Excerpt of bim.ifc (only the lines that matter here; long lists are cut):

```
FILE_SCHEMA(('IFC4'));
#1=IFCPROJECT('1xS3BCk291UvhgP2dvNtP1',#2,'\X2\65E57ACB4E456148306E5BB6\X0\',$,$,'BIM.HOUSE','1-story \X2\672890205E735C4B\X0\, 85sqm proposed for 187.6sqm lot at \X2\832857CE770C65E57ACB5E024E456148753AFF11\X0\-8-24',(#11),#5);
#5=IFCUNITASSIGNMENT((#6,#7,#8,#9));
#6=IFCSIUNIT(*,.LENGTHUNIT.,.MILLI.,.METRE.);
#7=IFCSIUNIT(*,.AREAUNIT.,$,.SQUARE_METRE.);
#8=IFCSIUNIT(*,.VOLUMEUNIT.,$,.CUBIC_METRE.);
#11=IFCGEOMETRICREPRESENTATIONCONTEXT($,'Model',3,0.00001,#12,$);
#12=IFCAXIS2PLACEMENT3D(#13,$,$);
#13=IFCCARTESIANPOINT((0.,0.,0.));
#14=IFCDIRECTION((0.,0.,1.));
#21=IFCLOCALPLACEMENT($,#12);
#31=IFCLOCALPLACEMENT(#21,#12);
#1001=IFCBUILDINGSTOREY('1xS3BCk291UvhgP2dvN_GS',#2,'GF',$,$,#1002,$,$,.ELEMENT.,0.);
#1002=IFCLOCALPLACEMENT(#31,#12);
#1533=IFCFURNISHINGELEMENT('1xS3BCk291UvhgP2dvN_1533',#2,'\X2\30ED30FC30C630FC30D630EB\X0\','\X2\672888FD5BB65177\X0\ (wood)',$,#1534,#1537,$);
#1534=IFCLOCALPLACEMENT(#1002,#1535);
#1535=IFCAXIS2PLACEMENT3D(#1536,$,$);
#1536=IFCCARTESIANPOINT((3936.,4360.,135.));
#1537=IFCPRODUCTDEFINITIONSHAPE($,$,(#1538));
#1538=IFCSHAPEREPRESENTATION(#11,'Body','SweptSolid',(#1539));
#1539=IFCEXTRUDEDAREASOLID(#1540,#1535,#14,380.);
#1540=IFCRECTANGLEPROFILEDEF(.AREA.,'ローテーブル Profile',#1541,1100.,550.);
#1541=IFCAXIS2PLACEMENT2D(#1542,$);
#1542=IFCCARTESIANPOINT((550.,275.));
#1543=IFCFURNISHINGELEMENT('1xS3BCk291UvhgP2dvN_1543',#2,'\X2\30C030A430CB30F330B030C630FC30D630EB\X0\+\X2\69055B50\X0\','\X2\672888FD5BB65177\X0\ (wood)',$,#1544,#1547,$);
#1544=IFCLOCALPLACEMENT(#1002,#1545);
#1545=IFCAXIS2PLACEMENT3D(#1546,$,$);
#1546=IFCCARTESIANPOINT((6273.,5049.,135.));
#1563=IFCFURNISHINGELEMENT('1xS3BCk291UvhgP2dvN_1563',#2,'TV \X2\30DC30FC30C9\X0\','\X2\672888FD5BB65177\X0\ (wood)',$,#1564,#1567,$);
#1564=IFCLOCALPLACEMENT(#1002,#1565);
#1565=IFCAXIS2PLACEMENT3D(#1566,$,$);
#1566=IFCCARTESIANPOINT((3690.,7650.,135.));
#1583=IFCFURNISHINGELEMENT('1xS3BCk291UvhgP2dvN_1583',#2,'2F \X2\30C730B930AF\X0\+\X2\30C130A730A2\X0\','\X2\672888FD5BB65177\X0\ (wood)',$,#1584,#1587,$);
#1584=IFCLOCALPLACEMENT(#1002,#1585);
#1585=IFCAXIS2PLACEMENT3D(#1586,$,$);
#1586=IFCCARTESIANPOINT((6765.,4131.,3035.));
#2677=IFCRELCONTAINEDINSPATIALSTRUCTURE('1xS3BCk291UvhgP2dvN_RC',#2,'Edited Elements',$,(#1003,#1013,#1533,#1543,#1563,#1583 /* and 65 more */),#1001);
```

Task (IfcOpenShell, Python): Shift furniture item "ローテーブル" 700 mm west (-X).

```python
import ifcopenshell
import ifcopenshell.api.geometry
import ifcopenshell.util.placement
import ifcopenshell.util.unit

model = ifcopenshell.open("bim.ifc")
unit_scale = ifcopenshell.util.unit.calculate_unit_scale(model)

item = model.by_guid("1xS3BCk291UvhgP2dvN_1533")
matrix = ifcopenshell.util.placement.get_local_placement(item.ObjectPlacement)
matrix[0, 3] -= 0.7 / unit_scale
ifcopenshell.api.geometry.edit_object_placement(model, product=item, matrix=matrix, is_si=False)

print(ifcopenshell.util.placement.get_local_placement(item.ObjectPlacement).round(3) + 0.0)

model.write("bim-out.ifc")
```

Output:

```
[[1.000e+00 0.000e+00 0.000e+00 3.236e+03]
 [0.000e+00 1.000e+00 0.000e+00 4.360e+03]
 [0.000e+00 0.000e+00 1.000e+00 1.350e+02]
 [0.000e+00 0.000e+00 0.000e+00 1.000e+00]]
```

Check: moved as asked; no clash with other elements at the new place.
